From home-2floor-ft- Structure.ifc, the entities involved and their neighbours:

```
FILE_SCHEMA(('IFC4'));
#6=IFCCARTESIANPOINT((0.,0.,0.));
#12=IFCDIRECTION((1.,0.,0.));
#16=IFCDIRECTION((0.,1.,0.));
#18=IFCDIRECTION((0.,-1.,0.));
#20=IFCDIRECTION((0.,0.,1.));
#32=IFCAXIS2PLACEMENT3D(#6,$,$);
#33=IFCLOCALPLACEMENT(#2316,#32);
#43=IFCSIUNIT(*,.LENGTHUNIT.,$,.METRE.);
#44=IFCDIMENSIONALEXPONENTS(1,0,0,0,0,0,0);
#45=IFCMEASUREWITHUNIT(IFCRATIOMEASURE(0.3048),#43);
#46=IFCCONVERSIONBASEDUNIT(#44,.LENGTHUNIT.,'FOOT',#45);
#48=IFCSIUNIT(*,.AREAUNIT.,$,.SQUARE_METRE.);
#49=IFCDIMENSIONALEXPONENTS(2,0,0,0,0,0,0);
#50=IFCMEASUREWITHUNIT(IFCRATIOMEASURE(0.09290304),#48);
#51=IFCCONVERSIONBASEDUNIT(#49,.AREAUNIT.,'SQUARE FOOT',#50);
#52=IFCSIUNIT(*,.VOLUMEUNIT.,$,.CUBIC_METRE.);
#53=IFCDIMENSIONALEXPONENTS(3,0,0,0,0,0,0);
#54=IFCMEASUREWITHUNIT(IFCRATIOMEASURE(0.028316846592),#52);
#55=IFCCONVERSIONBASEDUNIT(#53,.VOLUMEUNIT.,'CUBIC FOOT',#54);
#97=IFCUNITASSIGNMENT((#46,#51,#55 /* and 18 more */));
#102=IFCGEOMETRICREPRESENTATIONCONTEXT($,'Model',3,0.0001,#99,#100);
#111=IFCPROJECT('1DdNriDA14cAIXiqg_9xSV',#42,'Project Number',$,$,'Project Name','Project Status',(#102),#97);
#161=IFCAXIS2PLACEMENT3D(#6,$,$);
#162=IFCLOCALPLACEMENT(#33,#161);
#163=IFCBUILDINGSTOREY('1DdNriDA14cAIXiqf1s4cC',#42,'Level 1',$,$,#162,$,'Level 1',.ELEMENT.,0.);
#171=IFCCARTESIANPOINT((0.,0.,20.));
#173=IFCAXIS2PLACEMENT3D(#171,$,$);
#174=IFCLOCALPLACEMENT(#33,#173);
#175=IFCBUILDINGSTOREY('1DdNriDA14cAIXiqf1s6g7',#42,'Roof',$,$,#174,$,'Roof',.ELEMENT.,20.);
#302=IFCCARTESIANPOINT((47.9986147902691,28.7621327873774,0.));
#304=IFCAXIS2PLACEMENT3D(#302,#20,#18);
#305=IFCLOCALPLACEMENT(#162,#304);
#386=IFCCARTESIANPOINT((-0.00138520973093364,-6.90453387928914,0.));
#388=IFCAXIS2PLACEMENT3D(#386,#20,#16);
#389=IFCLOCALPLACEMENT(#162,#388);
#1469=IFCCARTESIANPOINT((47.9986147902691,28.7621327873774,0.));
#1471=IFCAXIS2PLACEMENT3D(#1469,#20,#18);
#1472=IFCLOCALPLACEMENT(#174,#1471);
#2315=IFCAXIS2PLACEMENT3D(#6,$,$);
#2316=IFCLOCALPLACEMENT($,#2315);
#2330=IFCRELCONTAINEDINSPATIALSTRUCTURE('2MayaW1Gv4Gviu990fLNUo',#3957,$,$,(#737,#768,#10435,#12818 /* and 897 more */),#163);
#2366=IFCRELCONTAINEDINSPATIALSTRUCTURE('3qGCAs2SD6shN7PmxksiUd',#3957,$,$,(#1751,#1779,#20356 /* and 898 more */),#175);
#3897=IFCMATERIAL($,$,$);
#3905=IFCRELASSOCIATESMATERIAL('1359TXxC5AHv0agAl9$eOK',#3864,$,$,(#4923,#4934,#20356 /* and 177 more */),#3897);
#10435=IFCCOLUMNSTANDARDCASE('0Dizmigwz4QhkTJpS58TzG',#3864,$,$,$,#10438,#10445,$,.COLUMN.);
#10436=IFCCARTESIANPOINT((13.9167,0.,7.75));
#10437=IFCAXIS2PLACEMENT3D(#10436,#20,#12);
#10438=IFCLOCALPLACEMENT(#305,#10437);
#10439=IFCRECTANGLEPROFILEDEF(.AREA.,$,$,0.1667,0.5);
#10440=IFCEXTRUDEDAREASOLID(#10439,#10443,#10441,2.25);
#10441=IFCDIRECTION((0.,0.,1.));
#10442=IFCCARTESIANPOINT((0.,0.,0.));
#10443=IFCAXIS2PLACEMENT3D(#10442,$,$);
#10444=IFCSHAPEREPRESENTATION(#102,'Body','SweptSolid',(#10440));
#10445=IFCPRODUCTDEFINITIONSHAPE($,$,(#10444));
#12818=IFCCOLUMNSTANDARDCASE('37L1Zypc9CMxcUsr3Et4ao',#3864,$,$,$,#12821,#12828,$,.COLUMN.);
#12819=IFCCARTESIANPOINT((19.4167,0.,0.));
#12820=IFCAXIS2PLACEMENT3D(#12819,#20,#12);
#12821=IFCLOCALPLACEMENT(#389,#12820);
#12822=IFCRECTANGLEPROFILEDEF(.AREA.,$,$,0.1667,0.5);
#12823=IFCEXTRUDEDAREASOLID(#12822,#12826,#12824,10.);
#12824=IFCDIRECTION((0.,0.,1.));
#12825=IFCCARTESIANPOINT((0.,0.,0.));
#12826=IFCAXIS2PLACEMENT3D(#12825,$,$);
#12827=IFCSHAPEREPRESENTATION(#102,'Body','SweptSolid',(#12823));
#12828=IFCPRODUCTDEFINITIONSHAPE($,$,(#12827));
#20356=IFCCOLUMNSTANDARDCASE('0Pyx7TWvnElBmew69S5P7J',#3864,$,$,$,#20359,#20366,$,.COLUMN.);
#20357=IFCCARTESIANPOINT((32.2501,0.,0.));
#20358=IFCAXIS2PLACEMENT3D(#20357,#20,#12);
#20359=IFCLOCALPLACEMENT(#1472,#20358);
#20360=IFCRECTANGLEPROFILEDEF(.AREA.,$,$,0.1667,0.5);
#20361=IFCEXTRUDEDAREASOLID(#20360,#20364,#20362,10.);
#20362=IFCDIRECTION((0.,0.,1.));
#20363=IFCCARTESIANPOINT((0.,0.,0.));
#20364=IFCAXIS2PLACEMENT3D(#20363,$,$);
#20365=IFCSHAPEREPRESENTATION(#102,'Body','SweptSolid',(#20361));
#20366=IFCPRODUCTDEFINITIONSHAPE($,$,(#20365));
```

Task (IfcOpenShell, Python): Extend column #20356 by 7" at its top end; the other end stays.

```python
import ifcopenshell
import ifcopenshell.util.unit

model = ifcopenshell.open("home-2floor-ft- Structure.ifc")
unit_scale = ifcopenshell.util.unit.calculate_unit_scale(model)

member = model.by_guid("0Pyx7TWvnElBmew69S5P7J")
change = 7 * 0.0254 / unit_scale

# The extrusion runs towards the end named, so only its depth changes.
body = next(r for r in member.Representation.Representations if r.RepresentationIdentifier == "Body")
solid = body.Items[0]
old_length = solid.Depth
solid.Depth += change

print(f"length {old_length:g} -> {solid.Depth:g}")

model.write("home-2floor-ft- Structure_updated.ifc")
```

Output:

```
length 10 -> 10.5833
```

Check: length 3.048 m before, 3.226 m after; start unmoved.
